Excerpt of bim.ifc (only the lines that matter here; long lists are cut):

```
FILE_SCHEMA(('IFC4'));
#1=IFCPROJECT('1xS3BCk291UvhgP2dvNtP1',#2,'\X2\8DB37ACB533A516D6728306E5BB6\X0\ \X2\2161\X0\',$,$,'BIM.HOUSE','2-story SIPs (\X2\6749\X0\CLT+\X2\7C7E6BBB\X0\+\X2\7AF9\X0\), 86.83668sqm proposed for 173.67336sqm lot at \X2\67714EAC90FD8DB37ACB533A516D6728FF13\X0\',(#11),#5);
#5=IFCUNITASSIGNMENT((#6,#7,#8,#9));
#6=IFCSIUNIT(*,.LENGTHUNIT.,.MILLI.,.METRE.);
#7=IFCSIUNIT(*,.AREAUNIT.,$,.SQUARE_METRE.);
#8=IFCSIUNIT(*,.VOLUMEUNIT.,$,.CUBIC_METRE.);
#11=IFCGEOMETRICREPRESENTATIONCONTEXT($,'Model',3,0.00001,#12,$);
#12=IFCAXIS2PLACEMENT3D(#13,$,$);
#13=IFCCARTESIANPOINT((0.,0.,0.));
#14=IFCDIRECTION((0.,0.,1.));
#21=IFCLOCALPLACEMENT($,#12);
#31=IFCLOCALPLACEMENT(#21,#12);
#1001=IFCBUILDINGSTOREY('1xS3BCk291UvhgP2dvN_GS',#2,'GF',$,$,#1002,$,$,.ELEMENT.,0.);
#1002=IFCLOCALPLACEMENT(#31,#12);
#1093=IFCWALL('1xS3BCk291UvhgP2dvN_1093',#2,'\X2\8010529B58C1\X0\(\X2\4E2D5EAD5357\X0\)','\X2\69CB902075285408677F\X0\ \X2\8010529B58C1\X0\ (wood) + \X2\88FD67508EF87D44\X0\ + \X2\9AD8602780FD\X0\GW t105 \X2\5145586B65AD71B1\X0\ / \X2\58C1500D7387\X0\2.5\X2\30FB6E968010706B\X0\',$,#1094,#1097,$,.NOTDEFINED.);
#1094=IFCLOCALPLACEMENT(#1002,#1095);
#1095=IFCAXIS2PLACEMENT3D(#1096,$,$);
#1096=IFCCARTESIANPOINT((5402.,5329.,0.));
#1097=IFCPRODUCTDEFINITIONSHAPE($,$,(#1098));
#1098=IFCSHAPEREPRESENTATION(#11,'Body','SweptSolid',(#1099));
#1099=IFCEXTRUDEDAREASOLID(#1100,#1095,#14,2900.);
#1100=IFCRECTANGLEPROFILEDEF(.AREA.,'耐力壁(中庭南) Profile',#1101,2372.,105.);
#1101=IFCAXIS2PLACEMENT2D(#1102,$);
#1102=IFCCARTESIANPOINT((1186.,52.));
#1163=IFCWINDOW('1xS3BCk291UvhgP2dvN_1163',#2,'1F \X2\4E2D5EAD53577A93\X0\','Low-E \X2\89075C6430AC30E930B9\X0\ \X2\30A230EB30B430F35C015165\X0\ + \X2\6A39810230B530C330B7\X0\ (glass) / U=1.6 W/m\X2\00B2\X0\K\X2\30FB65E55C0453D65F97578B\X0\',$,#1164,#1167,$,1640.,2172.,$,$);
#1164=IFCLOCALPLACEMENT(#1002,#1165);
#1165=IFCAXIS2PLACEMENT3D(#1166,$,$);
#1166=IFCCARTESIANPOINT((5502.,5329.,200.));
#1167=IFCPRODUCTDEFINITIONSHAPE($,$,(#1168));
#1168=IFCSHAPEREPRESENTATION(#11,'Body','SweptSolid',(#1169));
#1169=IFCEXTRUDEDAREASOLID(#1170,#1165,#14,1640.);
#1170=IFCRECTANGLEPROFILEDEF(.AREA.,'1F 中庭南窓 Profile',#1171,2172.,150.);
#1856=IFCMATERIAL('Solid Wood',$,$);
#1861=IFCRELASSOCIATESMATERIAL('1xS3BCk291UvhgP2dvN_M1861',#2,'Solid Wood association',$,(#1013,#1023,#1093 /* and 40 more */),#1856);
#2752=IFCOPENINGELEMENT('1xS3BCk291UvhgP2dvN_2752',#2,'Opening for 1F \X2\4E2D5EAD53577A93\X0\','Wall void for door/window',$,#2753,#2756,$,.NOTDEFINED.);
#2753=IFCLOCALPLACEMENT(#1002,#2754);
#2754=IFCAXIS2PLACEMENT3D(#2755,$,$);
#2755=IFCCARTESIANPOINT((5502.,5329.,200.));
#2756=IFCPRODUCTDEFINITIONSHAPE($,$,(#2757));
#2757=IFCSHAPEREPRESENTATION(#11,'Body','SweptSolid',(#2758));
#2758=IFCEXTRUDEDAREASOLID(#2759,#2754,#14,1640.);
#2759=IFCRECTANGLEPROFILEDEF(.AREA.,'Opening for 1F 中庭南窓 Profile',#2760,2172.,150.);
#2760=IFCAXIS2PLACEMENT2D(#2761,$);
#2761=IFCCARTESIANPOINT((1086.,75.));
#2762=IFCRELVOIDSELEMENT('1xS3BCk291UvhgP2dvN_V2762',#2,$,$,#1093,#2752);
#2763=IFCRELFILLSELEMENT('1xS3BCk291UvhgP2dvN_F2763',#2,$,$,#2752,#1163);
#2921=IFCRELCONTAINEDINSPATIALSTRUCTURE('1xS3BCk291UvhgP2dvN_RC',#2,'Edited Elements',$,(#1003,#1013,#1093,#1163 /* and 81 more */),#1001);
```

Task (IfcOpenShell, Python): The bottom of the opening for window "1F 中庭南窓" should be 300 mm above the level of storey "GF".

```python
import numpy as np
import ifcopenshell
import ifcopenshell.api.geometry
import ifcopenshell.geom
import ifcopenshell.util.element
import ifcopenshell.util.placement
import ifcopenshell.util.shape
import ifcopenshell.util.unit

model = ifcopenshell.open("bim.ifc")
unit_scale = ifcopenshell.util.unit.calculate_unit_scale(model)

window = model.by_id(1163)
opening = window.FillsVoids[0].RelatingOpeningElement
storey = ifcopenshell.util.element.get_container(window, ifc_class="IfcBuildingStorey")
level = ifcopenshell.util.placement.get_local_placement(storey.ObjectPlacement)[2, 3]

# The opening's origin need not be at the sill, so measure its lowest point.
shape = ifcopenshell.geom.create_shape(ifcopenshell.geom.settings(), opening)
bottom = ifcopenshell.util.shape.get_shape_bottom_elevation(shape, shape.geometry) / unit_scale
dz = level + 0.3 / unit_scale - bottom

shift = np.array([0.0, 0.0, dz])
# The window is not placed relative to its opening, so move both.
for product in (opening, window):
    matrix = ifcopenshell.util.placement.get_local_placement(product.ObjectPlacement)
    matrix[:3, 3] += shift
    ifcopenshell.api.geometry.edit_object_placement(model, product=product, matrix=matrix, is_si=False)

print(f"moved by {dz * unit_scale:+.3f} m")

model.write("bim_edited.ifc")
```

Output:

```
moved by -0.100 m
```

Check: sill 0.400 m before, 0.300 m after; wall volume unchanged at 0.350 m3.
